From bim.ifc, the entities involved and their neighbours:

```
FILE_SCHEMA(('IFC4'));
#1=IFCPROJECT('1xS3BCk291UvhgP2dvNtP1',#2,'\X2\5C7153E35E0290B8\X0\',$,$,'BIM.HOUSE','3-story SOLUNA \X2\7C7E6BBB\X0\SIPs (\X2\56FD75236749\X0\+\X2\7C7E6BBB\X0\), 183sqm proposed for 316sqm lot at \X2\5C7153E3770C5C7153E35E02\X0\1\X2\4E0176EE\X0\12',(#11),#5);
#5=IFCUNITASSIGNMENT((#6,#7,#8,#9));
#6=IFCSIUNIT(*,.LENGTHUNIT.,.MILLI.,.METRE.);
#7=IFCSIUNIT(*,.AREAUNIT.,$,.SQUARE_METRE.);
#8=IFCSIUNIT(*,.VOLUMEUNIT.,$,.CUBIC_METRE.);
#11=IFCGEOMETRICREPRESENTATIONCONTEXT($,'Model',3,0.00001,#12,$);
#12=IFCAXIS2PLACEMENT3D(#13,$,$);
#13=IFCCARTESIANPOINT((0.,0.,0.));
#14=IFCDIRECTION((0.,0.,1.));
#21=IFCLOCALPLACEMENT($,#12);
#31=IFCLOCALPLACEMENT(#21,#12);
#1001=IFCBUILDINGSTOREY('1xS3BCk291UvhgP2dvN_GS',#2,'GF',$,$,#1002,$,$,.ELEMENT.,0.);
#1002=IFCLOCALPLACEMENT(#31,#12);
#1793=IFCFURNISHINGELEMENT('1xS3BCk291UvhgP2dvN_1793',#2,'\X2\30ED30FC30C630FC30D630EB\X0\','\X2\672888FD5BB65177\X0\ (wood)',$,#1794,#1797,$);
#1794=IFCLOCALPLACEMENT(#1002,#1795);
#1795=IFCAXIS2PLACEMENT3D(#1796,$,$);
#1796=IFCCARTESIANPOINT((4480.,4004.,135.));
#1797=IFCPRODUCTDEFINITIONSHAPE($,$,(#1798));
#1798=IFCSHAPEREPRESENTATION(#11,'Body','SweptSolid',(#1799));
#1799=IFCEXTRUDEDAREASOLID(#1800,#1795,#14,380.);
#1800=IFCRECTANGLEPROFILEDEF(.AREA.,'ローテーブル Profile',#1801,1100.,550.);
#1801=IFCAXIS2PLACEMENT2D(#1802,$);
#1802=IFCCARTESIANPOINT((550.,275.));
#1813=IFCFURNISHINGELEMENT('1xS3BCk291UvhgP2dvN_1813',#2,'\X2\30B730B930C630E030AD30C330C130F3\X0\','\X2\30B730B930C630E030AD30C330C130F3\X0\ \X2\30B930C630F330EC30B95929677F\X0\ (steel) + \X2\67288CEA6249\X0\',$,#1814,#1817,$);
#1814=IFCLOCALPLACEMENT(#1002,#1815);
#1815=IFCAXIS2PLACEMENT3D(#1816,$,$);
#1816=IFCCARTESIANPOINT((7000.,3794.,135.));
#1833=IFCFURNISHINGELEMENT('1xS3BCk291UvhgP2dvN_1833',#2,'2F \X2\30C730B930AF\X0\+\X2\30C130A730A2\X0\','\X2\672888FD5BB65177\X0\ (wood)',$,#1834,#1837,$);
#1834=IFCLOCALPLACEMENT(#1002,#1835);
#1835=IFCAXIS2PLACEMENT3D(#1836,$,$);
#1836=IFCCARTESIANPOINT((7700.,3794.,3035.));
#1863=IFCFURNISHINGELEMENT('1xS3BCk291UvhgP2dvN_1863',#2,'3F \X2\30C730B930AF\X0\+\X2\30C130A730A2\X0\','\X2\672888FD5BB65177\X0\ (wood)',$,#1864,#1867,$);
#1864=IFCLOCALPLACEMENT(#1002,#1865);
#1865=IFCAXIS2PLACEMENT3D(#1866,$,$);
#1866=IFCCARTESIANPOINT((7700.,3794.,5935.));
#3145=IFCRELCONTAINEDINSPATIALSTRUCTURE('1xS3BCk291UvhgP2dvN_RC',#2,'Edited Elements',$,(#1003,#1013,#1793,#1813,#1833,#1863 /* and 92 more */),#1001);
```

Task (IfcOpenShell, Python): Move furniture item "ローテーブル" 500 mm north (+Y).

```python
import ifcopenshell
import ifcopenshell.api.geometry
import ifcopenshell.util.placement

model = ifcopenshell.open("bim.ifc")

item = model.by_guid("1xS3BCk291UvhgP2dvN_1793")
matrix = ifcopenshell.util.placement.get_local_placement(item.ObjectPlacement)
matrix[1, 3] += 500.0
ifcopenshell.api.geometry.edit_object_placement(model, product=item, matrix=matrix, is_si=False)

print(ifcopenshell.util.placement.get_local_placement(item.ObjectPlacement).round(3) + 0.0)

model.write("bim_v2.ifc")
```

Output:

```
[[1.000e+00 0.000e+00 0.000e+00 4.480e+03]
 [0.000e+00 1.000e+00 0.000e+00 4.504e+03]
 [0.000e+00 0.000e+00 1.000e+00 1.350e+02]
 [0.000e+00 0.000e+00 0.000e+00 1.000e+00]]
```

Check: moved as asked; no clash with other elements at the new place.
